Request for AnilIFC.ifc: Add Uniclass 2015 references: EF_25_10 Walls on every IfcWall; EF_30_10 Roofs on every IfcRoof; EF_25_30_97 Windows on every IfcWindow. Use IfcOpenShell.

First a look at what the model holds.

```python
import ifcopenshell

model = ifcopenshell.open("AnilIFC.ifc")
print(model.schema)
print("classifications:", [c.Name for c in model.by_type("IfcClassification")])
for ifc_class in ("IfcDoor", "IfcRoof", "IfcStair", "IfcWall", "IfcWindow"):
    print(ifc_class, len(model.by_type(ifc_class)))
```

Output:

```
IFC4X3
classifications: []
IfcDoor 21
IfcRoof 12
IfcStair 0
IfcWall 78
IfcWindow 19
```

```python
import ifcopenshell
import ifcopenshell.api.classification

model = ifcopenshell.open("AnilIFC.ifc")

system = ifcopenshell.api.classification.add_classification(model, classification="Uniclass 2015")

codes = {
    "IfcWall": ("EF_25_10", "Walls"),
    "IfcRoof": ("EF_30_10", "Roofs"),
    "IfcWindow": ("EF_25_30_97", "Windows"),
}
for ifc_class, (code, name) in codes.items():
    products = model.by_type(ifc_class)
    ifcopenshell.api.classification.add_reference(
        model, products=products, classification=system, identification=code, name=name
    )
    print(code, len(products))

model.write("AnilIFC-out.ifc")
```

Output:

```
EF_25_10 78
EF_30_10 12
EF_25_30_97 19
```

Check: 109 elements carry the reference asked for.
